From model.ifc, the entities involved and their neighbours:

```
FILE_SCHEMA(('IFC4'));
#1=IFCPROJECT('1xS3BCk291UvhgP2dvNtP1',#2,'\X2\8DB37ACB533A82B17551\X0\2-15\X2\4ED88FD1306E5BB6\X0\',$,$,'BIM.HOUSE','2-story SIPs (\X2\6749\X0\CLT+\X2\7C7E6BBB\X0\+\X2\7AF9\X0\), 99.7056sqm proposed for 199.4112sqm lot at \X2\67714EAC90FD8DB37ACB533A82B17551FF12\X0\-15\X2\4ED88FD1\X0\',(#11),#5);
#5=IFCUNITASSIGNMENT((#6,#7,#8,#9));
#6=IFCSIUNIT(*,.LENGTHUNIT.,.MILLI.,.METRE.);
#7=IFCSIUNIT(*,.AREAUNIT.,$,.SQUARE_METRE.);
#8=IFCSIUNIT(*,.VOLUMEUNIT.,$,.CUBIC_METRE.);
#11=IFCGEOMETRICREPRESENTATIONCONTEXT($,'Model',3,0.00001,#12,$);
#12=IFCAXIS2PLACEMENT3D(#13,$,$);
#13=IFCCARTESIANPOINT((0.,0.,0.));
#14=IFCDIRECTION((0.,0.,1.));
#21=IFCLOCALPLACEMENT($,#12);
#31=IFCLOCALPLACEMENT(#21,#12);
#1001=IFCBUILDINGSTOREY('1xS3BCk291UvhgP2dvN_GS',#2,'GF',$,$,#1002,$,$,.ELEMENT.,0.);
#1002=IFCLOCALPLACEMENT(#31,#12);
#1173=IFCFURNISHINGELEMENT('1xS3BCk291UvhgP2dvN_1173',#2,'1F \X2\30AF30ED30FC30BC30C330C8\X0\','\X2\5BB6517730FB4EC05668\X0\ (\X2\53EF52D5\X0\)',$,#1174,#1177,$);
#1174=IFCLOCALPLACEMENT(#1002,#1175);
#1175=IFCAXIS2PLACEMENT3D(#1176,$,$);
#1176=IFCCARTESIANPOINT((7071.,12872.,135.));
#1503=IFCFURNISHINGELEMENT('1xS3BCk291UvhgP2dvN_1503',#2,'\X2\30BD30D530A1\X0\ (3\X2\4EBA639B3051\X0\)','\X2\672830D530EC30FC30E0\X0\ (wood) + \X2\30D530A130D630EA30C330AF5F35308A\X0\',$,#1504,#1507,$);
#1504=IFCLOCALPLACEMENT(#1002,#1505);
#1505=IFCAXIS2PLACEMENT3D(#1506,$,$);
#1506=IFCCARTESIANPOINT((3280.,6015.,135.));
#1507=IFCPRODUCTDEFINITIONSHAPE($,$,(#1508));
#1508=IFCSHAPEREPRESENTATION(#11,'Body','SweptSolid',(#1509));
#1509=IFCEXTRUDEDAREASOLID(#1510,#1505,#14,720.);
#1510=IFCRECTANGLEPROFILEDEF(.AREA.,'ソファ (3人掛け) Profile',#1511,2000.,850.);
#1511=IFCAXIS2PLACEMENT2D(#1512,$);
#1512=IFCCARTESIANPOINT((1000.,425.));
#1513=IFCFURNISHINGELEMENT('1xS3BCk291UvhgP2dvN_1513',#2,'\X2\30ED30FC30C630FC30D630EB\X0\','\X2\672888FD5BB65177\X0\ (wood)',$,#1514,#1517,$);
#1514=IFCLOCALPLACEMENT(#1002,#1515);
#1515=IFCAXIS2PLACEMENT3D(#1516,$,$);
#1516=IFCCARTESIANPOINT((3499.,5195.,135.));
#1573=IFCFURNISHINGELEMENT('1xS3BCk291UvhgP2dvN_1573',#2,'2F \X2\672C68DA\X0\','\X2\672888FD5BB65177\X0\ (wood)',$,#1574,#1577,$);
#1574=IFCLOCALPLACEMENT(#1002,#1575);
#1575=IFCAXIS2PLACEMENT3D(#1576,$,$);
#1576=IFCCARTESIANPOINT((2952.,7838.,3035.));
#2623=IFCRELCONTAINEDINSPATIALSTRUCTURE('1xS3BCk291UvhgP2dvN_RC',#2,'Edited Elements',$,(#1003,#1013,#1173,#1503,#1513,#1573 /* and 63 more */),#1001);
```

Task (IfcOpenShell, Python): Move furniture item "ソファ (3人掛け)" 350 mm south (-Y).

```python
import ifcopenshell
import ifcopenshell.api.geometry
import ifcopenshell.util.placement
import ifcopenshell.util.unit

model = ifcopenshell.open("model.ifc")
unit_scale = ifcopenshell.util.unit.calculate_unit_scale(model)

item = model.by_guid("1xS3BCk291UvhgP2dvN_1503")
matrix = ifcopenshell.util.placement.get_local_placement(item.ObjectPlacement)
matrix[1, 3] -= 0.35 / unit_scale
ifcopenshell.api.geometry.edit_object_placement(model, product=item, matrix=matrix, is_si=False)

print(ifcopenshell.util.placement.get_local_placement(item.ObjectPlacement).round(3) + 0.0)

model.write("model_updated.ifc")
```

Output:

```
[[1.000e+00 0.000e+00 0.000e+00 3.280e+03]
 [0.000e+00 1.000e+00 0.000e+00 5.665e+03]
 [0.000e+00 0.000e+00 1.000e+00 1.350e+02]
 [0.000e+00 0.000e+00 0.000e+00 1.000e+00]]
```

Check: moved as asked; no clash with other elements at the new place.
